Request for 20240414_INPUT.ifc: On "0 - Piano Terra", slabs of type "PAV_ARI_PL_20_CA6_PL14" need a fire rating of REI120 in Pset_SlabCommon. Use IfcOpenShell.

First a look at what the model holds.

```python
import ifcopenshell
import ifcopenshell.util.element

model = ifcopenshell.open("20240414_INPUT.ifc")
print(model.schema)
storey = next(s for s in model.by_type("IfcBuildingStorey") if s.Name == "0 - Piano Terra")
slabs = [e for e in ifcopenshell.util.element.get_decomposition(storey) if e.is_a("IfcSlab")]
seen = {}
for e in slabs:
    element_type = ifcopenshell.util.element.get_type(e)
    key = (element_type.Name if element_type != e and element_type else None, ifcopenshell.util.element.get_pset(e, "Pset_SlabCommon", "FireRating"))
    seen[key] = seen.get(key, 0) + 1
for (name, value), count in sorted(seen.items(), key=str):
    print(count, "x", name, "|", value)
```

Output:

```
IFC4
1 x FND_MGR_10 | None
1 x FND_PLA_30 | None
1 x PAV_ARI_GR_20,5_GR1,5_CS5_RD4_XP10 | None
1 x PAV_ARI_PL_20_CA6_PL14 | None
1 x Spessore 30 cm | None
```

```python
import ifcopenshell
import ifcopenshell.api.pset
import ifcopenshell.util.element

model = ifcopenshell.open("20240414_INPUT.ifc")

storey = next(s for s in model.by_type("IfcBuildingStorey") if s.Name == "0 - Piano Terra")
slabs = [e for e in ifcopenshell.util.element.get_decomposition(storey) if e.is_a("IfcSlab")]

count = 0
for e in slabs:
    element_type = ifcopenshell.util.element.get_type(e)
    if element_type in (None, e) or element_type.Name != "PAV_ARI_PL_20_CA6_PL14":
        continue
    # add_pset returns the element's existing set when there is one.
    pset = ifcopenshell.api.pset.add_pset(model, product=e, name="Pset_SlabCommon")
    ifcopenshell.api.pset.edit_pset(model, pset=pset, properties={"FireRating": "REI120"})
    count += 1

print(count, "slabs updated")

model.write("20240414_INPUT-out.ifc")
```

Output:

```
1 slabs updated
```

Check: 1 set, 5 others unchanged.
